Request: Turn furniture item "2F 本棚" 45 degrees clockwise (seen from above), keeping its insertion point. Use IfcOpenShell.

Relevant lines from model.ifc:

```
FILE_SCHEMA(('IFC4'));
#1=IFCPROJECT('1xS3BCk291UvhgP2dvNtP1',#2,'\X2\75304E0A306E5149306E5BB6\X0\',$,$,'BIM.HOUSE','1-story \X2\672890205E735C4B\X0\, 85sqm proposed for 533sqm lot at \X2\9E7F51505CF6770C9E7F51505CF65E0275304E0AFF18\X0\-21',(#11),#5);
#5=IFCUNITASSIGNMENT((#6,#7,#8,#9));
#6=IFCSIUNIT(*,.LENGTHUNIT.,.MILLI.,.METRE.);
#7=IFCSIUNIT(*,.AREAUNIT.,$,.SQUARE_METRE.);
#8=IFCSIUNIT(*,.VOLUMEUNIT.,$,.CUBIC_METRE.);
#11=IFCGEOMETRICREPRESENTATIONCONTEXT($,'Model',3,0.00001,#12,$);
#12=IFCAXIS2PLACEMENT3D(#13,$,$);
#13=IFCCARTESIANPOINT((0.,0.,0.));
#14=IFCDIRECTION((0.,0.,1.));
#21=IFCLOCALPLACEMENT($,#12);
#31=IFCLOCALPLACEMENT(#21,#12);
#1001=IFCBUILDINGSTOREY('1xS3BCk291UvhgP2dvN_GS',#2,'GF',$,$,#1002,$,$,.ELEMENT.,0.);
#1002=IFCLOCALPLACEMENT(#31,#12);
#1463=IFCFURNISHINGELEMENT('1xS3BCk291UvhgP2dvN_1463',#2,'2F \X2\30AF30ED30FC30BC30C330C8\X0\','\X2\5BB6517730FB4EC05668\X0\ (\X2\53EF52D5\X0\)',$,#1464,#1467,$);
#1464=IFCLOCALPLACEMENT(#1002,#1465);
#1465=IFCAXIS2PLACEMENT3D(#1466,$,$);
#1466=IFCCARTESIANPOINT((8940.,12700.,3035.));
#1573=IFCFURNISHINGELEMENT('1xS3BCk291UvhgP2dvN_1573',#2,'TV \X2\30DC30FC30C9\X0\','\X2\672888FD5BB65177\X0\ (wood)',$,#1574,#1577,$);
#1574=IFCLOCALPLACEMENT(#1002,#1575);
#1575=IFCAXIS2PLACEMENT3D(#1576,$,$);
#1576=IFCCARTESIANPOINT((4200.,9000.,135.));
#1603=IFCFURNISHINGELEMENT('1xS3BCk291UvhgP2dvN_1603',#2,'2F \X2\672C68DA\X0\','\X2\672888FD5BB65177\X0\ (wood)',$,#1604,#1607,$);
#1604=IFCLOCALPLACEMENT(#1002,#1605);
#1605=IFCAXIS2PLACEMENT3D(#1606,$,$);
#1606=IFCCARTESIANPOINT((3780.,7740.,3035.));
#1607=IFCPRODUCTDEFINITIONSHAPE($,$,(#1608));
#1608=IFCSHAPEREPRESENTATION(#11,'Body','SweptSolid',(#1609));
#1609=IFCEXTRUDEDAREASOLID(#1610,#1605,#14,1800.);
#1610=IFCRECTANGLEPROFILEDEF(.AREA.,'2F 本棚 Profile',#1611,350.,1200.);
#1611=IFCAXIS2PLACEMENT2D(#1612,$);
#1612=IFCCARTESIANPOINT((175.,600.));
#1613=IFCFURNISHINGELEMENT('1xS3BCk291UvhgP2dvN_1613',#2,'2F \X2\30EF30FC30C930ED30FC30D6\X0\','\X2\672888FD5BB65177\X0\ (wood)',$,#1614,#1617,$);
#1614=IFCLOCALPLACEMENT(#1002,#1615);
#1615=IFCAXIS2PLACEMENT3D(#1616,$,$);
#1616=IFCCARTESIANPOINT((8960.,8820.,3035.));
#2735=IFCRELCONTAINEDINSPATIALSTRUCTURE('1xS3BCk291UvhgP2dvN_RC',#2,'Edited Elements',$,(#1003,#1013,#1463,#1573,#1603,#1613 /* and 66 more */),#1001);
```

```python
import ifcopenshell
import ifcopenshell.api.geometry
import ifcopenshell.util.placement

model = ifcopenshell.open("model.ifc")

item = model.by_guid("1xS3BCk291UvhgP2dvN_1603")
matrix = ifcopenshell.util.placement.get_local_placement(item.ObjectPlacement)
matrix = matrix @ ifcopenshell.util.placement.rotation(-45, "Z")
ifcopenshell.api.geometry.edit_object_placement(model, product=item, matrix=matrix, is_si=False)

print(ifcopenshell.util.placement.get_local_placement(item.ObjectPlacement).round(3) + 0.0)

model.write("model-out.ifc")
```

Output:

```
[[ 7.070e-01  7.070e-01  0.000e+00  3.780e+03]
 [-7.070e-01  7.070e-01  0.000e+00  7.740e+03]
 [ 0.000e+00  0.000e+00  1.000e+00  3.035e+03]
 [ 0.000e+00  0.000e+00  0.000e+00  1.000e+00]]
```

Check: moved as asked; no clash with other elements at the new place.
